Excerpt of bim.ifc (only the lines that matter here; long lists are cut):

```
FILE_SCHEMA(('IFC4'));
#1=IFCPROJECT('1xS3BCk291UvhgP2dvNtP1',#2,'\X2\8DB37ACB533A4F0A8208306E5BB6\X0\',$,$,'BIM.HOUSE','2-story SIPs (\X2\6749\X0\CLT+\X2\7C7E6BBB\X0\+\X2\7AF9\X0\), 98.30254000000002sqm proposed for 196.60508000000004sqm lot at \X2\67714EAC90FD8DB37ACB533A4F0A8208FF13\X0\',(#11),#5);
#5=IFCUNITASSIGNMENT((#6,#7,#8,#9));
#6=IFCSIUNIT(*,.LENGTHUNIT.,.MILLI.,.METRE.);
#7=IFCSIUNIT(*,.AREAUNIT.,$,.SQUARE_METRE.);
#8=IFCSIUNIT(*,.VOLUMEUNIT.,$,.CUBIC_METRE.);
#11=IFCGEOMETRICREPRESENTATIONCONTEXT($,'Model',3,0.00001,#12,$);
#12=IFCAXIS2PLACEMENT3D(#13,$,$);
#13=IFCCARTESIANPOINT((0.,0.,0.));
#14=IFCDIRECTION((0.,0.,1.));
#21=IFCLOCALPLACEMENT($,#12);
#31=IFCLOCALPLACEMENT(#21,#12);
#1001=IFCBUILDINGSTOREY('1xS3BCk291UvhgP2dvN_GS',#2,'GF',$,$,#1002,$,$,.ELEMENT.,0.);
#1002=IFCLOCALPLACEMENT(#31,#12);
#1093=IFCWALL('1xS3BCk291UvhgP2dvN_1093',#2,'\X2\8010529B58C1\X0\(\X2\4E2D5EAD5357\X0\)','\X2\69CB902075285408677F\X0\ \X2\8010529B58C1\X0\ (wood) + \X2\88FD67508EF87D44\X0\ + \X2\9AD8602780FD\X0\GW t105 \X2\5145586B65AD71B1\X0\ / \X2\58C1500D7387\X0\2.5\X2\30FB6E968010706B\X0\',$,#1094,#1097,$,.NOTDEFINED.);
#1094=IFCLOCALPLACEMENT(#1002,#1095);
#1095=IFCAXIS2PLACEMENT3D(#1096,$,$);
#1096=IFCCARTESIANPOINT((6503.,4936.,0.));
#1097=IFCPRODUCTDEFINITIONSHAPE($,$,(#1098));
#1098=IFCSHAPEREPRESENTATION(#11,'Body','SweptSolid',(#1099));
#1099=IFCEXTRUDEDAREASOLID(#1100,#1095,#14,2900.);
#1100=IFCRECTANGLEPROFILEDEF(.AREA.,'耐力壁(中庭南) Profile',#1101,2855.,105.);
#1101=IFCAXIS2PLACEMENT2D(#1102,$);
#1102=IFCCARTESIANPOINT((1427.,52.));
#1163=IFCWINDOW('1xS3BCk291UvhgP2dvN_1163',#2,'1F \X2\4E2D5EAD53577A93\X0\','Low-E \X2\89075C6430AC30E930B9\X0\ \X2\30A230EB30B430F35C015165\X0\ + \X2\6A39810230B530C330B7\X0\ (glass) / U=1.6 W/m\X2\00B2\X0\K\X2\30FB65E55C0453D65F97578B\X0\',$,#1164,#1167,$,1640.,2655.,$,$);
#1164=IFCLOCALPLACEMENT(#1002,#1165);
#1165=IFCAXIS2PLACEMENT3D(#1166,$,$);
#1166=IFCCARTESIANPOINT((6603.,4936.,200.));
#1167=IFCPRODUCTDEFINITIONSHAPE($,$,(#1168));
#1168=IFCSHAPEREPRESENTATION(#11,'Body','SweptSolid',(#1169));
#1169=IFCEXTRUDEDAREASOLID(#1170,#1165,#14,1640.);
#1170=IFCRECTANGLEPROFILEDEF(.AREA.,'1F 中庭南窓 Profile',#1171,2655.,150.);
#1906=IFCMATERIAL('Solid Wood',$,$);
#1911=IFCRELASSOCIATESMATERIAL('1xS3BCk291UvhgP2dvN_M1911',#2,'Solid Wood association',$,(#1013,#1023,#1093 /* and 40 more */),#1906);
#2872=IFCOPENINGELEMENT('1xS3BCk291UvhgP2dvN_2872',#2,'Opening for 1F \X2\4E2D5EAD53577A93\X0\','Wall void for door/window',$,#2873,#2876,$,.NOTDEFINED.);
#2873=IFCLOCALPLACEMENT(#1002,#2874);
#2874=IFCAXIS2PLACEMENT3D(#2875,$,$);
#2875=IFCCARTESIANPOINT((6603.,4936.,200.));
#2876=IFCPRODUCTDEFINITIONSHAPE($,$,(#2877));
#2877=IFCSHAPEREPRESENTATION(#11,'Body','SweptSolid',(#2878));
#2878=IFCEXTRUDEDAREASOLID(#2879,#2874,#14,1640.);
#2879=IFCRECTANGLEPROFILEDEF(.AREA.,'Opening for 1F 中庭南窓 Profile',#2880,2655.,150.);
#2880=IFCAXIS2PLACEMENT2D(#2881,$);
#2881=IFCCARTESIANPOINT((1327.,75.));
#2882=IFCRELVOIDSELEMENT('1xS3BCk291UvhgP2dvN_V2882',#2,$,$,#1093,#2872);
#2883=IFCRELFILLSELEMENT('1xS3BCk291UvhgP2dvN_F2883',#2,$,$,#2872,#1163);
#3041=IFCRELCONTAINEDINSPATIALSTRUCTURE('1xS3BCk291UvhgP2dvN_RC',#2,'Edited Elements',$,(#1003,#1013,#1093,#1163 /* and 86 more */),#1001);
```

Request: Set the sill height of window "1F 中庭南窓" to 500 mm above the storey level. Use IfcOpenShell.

```python
import numpy as np
import ifcopenshell
import ifcopenshell.api.geometry
import ifcopenshell.geom
import ifcopenshell.util.element
import ifcopenshell.util.placement
import ifcopenshell.util.shape
import ifcopenshell.util.unit

model = ifcopenshell.open("bim.ifc")
unit_scale = ifcopenshell.util.unit.calculate_unit_scale(model)

window = model.by_guid("1xS3BCk291UvhgP2dvN_1163")
opening = window.FillsVoids[0].RelatingOpeningElement
storey = ifcopenshell.util.element.get_container(window, ifc_class="IfcBuildingStorey")
level = ifcopenshell.util.placement.get_local_placement(storey.ObjectPlacement)[2, 3]

# The opening's origin need not be at the sill, so measure its lowest point.
shape = ifcopenshell.geom.create_shape(ifcopenshell.geom.settings(), opening)
bottom = ifcopenshell.util.shape.get_shape_bottom_elevation(shape, shape.geometry) / unit_scale
dz = level + 0.5 / unit_scale - bottom

shift = np.array([0.0, 0.0, dz])
# The window is not placed relative to its opening, so move both.
for product in (opening, window):
    matrix = ifcopenshell.util.placement.get_local_placement(product.ObjectPlacement)
    matrix[:3, 3] += shift
    ifcopenshell.api.geometry.edit_object_placement(model, product=product, matrix=matrix, is_si=False)

print(f"moved by {dz * unit_scale:+.3f} m")

model.write("bim_v2.ifc")
```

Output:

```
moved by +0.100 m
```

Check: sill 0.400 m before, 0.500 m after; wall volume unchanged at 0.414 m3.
